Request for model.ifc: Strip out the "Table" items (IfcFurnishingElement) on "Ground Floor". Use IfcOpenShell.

First a look at what the model holds.

```python
import ifcopenshell
import ifcopenshell.util.element

model = ifcopenshell.open("model.ifc")
print(model.schema)
storey = next(s for s in model.by_type("IfcBuildingStorey") if s.Name == "Ground Floor")
furniture = [e for e in ifcopenshell.util.element.get_decomposition(storey) if e.is_a("IfcFurnishingElement")]
seen = {}
for e in furniture:
    element_type = ifcopenshell.util.element.get_type(e)
    name = element_type.Name if element_type not in (None, e) else None
    seen[name] = seen.get(name, 0) + 1
for name, count in sorted(seen.items(), key=str):
    print(count, "x", name)
```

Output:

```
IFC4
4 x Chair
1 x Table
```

```python
import ifcopenshell
import ifcopenshell.api.root
import ifcopenshell.util.element

model = ifcopenshell.open("model.ifc")

storey = next(s for s in model.by_type("IfcBuildingStorey") if s.Name == "Ground Floor")
furniture = [e for e in ifcopenshell.util.element.get_decomposition(storey) if e.is_a("IfcFurnishingElement")]
targets = [e for e in furniture if (t := ifcopenshell.util.element.get_type(e)) not in (None, e) and t.Name == "Table"]

for e in targets:
    ifcopenshell.api.root.remove_product(model, product=e)
print(len(targets), "removed")

model.write("model_v2.ifc")
```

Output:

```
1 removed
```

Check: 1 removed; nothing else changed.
